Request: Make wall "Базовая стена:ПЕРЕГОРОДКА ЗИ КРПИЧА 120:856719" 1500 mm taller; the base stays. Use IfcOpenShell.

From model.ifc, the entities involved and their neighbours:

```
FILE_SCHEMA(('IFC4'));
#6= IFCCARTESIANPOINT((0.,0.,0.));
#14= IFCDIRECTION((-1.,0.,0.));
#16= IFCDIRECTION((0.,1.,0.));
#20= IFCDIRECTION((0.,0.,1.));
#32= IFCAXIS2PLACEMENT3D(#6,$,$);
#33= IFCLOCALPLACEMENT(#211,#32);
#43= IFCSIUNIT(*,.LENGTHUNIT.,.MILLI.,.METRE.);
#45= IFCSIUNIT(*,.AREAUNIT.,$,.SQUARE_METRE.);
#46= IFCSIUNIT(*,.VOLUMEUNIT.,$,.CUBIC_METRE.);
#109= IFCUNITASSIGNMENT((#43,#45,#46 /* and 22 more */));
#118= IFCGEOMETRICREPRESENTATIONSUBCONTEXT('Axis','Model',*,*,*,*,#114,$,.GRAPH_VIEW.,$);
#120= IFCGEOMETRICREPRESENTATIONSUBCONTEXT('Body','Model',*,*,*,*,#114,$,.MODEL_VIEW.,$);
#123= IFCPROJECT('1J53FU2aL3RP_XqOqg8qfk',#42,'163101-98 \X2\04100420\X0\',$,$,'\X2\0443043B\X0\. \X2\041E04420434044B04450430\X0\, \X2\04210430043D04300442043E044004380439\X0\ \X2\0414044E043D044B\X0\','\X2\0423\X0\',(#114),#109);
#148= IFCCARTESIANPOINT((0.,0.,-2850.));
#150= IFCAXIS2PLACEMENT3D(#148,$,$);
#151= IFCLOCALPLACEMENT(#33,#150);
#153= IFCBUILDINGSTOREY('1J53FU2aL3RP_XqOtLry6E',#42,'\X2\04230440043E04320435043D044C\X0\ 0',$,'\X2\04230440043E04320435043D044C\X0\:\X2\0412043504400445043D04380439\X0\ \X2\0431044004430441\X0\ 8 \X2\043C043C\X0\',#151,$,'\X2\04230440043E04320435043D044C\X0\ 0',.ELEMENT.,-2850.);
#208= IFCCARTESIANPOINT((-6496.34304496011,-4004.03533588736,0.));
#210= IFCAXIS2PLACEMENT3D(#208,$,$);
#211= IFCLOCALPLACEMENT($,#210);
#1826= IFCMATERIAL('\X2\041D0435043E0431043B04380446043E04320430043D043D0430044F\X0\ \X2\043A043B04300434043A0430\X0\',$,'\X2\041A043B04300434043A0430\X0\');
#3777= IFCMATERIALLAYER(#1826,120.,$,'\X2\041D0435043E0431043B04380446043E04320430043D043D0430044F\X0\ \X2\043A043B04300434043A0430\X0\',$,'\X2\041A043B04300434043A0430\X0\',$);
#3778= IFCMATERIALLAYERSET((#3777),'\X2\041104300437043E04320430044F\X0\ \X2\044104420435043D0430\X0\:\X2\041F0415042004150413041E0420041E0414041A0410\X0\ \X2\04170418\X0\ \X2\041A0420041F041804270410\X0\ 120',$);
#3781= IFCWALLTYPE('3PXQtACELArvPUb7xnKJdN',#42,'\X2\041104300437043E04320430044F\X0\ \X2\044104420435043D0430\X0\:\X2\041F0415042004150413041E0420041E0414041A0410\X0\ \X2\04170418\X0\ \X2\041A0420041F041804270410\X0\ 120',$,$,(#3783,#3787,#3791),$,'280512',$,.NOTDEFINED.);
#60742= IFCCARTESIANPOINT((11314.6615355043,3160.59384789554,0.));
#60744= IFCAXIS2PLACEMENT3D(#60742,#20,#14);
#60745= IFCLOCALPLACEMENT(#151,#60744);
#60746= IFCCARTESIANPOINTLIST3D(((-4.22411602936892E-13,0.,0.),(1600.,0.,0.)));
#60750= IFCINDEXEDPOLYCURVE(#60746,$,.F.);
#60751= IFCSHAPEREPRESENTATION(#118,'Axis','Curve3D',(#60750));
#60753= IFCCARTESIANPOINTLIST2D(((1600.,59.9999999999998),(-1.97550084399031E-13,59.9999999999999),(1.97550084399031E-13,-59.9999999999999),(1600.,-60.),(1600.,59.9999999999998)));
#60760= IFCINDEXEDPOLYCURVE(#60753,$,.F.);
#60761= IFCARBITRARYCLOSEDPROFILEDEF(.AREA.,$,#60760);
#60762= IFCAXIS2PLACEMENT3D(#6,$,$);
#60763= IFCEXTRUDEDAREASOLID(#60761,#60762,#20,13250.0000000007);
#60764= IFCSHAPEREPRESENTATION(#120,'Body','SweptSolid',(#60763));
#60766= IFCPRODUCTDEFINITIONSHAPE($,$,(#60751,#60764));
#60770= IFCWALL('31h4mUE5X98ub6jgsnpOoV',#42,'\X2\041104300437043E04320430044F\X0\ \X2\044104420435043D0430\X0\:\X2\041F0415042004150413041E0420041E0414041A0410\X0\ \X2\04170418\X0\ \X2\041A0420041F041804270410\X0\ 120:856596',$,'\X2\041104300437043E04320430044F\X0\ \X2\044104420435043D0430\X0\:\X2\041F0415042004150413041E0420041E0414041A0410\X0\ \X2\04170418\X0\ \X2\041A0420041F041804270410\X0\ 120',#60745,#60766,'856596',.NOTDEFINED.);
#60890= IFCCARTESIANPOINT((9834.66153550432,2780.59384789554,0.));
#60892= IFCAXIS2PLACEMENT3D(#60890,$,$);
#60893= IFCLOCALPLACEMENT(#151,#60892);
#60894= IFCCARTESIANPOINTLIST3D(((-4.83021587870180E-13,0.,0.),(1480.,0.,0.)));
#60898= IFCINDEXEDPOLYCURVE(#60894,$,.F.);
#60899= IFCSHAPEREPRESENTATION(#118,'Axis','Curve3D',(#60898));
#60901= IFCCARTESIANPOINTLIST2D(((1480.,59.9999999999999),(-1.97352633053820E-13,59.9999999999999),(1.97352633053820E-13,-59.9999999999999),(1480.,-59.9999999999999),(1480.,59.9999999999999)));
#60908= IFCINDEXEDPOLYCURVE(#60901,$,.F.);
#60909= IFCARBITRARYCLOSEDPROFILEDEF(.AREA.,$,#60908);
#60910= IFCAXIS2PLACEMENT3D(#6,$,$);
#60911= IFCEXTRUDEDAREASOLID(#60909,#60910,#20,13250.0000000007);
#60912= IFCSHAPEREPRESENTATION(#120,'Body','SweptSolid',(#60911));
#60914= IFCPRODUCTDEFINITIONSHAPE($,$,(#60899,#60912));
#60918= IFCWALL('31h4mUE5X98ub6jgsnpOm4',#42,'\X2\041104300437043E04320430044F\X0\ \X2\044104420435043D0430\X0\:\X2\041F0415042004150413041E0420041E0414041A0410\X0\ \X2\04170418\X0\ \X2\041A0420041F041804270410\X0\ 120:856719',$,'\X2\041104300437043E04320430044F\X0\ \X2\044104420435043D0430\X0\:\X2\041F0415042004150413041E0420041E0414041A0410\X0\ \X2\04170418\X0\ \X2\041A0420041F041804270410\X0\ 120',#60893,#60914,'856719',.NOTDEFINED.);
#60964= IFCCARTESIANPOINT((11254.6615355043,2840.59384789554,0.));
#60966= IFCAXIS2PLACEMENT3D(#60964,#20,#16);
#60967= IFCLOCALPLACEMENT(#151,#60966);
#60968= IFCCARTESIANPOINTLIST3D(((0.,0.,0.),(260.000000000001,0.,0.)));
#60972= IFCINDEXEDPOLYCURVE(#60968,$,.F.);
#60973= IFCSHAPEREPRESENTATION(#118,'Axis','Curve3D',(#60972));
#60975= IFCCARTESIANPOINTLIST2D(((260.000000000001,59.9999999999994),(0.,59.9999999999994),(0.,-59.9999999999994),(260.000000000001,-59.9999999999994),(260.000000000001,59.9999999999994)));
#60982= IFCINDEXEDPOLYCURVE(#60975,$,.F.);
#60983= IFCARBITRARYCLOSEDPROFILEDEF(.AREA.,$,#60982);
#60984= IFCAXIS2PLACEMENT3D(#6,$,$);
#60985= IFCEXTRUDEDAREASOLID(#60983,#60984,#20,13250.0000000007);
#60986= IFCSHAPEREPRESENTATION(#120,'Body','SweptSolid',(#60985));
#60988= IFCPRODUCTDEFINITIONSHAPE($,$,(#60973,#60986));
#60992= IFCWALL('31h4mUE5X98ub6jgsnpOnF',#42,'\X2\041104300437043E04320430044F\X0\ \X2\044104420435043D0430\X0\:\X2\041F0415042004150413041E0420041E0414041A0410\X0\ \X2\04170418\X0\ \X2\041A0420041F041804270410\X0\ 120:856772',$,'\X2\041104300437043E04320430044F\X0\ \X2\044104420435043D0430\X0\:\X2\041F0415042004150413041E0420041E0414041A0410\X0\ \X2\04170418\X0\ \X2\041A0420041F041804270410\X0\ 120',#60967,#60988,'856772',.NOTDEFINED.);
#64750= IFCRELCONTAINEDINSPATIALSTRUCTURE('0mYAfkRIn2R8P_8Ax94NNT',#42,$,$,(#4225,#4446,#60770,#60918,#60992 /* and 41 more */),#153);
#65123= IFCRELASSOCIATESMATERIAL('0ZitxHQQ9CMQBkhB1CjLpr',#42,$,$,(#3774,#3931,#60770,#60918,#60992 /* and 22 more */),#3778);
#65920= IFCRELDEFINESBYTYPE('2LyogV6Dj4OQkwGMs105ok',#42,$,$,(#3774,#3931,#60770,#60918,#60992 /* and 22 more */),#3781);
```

```python
import ifcopenshell
import ifcopenshell.geom
import ifcopenshell.util.representation
import ifcopenshell.util.shape

model = ifcopenshell.open("model.ifc")
settings = ifcopenshell.geom.settings()


def volume(element):
    """Net volume in cubic metres, openings subtracted."""
    shape = ifcopenshell.geom.create_shape(settings, element)
    return ifcopenshell.util.shape.get_volume(shape.geometry)


wall = model.by_id(60918)
before = volume(wall)

body = ifcopenshell.util.representation.get_representation(wall, "Model", "Body")
solid = body.Items[0]
old_height = solid.Depth
solid.Depth += 1500.0
after = volume(wall)

print(f"height {old_height:g} -> {solid.Depth:g}, volume {before:.3f} -> {after:.3f} m3")

model.write("model-out.ifc")
```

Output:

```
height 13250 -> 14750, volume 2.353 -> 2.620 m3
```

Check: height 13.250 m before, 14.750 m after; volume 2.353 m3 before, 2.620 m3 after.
